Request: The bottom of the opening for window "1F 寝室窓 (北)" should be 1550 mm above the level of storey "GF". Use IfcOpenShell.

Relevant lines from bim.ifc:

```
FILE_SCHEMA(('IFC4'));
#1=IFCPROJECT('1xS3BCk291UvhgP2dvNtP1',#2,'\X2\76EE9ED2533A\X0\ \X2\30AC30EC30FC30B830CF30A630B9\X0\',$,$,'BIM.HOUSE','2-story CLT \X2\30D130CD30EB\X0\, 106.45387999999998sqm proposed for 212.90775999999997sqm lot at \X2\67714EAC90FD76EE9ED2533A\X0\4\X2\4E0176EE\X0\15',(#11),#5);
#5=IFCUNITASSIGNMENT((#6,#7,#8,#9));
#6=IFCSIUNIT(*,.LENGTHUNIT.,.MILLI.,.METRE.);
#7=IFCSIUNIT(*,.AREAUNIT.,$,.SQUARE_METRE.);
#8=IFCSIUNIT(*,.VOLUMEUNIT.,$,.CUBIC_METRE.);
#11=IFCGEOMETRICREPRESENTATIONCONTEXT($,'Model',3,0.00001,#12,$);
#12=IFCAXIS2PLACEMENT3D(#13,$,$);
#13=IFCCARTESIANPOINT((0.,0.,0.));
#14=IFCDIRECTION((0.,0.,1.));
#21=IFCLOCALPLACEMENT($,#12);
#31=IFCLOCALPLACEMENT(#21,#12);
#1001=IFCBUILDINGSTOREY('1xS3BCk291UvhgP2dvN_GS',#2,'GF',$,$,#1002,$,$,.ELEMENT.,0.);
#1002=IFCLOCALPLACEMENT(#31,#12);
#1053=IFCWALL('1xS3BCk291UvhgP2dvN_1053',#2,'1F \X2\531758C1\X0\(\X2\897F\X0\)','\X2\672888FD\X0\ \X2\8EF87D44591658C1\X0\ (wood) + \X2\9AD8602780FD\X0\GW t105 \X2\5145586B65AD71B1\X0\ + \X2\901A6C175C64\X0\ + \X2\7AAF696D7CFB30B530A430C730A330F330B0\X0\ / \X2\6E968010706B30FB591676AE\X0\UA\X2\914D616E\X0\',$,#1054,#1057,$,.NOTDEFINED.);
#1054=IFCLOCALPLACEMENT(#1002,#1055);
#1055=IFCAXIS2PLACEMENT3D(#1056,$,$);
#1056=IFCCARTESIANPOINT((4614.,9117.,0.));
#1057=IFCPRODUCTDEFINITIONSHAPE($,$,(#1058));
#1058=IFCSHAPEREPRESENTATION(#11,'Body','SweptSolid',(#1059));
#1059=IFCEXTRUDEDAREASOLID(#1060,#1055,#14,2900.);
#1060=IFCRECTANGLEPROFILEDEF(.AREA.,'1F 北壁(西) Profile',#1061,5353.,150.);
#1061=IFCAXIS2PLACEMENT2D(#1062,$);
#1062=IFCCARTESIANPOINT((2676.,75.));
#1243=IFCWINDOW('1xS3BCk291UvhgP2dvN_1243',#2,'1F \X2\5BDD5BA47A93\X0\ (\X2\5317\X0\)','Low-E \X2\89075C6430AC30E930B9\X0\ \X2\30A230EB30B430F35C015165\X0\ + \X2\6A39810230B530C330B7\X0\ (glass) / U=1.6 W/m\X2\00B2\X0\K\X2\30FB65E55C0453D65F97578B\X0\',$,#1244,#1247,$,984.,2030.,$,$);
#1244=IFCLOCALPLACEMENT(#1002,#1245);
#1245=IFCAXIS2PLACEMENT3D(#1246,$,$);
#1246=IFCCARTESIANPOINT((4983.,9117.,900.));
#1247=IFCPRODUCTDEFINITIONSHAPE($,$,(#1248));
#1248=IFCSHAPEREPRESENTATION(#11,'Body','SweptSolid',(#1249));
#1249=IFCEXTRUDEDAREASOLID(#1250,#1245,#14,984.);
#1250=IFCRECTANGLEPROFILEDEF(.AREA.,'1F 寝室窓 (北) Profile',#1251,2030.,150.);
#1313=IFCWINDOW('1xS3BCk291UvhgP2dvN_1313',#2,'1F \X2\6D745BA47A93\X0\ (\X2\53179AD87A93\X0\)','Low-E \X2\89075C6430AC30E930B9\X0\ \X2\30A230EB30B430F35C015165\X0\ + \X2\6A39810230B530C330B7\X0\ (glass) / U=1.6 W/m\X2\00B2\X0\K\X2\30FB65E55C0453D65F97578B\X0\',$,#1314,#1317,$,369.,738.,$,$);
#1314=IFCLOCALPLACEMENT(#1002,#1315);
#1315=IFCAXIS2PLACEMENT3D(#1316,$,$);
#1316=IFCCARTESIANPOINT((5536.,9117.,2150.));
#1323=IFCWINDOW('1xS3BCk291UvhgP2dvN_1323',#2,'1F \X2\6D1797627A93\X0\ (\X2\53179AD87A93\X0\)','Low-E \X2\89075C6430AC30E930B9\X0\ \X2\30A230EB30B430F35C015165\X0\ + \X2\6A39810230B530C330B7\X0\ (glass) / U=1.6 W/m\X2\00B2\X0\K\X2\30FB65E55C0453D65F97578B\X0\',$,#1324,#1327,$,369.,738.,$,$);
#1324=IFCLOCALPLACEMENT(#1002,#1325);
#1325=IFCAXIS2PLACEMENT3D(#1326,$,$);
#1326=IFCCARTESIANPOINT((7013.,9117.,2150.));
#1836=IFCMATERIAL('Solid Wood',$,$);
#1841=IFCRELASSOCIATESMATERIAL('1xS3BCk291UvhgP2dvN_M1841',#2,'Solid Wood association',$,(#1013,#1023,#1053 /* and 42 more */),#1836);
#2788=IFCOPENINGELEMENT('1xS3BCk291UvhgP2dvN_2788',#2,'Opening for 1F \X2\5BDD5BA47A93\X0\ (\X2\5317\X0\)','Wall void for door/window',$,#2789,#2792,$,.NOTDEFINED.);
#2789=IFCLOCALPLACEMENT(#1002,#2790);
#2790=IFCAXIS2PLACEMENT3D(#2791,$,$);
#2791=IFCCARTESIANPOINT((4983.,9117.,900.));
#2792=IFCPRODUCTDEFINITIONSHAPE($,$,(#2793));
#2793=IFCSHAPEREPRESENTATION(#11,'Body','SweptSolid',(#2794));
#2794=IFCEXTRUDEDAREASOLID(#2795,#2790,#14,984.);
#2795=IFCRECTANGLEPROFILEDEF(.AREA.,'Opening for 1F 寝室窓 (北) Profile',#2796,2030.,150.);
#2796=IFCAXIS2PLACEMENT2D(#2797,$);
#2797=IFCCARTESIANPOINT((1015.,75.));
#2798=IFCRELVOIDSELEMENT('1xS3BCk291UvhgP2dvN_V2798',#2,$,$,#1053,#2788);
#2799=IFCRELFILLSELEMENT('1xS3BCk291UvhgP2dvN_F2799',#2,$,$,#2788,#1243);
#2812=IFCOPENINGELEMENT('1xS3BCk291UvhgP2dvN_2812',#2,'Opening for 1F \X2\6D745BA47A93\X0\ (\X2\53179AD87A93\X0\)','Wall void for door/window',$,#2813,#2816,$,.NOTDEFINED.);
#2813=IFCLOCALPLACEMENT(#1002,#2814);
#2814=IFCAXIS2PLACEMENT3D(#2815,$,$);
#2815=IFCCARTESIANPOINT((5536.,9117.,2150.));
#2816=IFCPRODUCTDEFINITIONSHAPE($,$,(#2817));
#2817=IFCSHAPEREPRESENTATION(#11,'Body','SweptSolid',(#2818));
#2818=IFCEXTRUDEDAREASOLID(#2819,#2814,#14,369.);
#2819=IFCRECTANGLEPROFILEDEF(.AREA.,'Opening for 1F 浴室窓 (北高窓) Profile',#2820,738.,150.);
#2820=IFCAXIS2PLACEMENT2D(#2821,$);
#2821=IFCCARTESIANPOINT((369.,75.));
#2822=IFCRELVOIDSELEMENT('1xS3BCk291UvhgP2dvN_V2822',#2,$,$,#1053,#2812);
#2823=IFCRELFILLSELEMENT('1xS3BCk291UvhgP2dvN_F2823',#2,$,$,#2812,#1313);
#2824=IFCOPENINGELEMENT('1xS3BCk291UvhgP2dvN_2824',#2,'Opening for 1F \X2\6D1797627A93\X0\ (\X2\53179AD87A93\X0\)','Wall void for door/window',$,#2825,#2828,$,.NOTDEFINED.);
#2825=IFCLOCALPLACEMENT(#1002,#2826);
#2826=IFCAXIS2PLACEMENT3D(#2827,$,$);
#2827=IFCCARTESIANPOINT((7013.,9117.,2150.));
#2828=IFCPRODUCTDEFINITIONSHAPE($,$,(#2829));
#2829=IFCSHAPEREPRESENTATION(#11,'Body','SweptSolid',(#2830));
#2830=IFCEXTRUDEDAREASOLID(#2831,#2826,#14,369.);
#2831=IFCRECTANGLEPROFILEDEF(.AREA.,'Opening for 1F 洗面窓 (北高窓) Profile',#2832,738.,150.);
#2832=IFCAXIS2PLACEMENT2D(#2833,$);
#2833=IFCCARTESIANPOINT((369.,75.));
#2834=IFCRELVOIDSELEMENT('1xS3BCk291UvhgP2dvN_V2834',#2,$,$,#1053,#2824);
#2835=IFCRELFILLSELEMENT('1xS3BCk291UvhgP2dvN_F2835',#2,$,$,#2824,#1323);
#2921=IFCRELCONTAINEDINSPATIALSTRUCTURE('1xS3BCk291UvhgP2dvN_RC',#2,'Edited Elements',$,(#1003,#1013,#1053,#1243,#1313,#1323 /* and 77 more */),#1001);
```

```python
import numpy as np
import ifcopenshell
import ifcopenshell.api.geometry
import ifcopenshell.geom
import ifcopenshell.util.element
import ifcopenshell.util.placement
import ifcopenshell.util.shape
import ifcopenshell.util.unit

model = ifcopenshell.open("bim.ifc")
unit_scale = ifcopenshell.util.unit.calculate_unit_scale(model)

window = model.by_guid("1xS3BCk291UvhgP2dvN_1243")
opening = window.FillsVoids[0].RelatingOpeningElement
storey = ifcopenshell.util.element.get_container(window, ifc_class="IfcBuildingStorey")
level = ifcopenshell.util.placement.get_local_placement(storey.ObjectPlacement)[2, 3]

# The opening's origin need not be at the sill, so measure its lowest point.
shape = ifcopenshell.geom.create_shape(ifcopenshell.geom.settings(), opening)
bottom = ifcopenshell.util.shape.get_shape_bottom_elevation(shape, shape.geometry) / unit_scale
dz = level + 1550.0 - bottom

shift = np.array([0.0, 0.0, dz])
# The window is not placed relative to its opening, so move both.
for product in (opening, window):
    matrix = ifcopenshell.util.placement.get_local_placement(product.ObjectPlacement)
    matrix[:3, 3] += shift
    ifcopenshell.api.geometry.edit_object_placement(model, product=product, matrix=matrix, is_si=False)

print(f"moved by {dz * unit_scale:+.3f} m")

model.write("bim_edited.ifc")
```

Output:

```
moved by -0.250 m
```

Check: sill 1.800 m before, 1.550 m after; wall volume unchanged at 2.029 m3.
